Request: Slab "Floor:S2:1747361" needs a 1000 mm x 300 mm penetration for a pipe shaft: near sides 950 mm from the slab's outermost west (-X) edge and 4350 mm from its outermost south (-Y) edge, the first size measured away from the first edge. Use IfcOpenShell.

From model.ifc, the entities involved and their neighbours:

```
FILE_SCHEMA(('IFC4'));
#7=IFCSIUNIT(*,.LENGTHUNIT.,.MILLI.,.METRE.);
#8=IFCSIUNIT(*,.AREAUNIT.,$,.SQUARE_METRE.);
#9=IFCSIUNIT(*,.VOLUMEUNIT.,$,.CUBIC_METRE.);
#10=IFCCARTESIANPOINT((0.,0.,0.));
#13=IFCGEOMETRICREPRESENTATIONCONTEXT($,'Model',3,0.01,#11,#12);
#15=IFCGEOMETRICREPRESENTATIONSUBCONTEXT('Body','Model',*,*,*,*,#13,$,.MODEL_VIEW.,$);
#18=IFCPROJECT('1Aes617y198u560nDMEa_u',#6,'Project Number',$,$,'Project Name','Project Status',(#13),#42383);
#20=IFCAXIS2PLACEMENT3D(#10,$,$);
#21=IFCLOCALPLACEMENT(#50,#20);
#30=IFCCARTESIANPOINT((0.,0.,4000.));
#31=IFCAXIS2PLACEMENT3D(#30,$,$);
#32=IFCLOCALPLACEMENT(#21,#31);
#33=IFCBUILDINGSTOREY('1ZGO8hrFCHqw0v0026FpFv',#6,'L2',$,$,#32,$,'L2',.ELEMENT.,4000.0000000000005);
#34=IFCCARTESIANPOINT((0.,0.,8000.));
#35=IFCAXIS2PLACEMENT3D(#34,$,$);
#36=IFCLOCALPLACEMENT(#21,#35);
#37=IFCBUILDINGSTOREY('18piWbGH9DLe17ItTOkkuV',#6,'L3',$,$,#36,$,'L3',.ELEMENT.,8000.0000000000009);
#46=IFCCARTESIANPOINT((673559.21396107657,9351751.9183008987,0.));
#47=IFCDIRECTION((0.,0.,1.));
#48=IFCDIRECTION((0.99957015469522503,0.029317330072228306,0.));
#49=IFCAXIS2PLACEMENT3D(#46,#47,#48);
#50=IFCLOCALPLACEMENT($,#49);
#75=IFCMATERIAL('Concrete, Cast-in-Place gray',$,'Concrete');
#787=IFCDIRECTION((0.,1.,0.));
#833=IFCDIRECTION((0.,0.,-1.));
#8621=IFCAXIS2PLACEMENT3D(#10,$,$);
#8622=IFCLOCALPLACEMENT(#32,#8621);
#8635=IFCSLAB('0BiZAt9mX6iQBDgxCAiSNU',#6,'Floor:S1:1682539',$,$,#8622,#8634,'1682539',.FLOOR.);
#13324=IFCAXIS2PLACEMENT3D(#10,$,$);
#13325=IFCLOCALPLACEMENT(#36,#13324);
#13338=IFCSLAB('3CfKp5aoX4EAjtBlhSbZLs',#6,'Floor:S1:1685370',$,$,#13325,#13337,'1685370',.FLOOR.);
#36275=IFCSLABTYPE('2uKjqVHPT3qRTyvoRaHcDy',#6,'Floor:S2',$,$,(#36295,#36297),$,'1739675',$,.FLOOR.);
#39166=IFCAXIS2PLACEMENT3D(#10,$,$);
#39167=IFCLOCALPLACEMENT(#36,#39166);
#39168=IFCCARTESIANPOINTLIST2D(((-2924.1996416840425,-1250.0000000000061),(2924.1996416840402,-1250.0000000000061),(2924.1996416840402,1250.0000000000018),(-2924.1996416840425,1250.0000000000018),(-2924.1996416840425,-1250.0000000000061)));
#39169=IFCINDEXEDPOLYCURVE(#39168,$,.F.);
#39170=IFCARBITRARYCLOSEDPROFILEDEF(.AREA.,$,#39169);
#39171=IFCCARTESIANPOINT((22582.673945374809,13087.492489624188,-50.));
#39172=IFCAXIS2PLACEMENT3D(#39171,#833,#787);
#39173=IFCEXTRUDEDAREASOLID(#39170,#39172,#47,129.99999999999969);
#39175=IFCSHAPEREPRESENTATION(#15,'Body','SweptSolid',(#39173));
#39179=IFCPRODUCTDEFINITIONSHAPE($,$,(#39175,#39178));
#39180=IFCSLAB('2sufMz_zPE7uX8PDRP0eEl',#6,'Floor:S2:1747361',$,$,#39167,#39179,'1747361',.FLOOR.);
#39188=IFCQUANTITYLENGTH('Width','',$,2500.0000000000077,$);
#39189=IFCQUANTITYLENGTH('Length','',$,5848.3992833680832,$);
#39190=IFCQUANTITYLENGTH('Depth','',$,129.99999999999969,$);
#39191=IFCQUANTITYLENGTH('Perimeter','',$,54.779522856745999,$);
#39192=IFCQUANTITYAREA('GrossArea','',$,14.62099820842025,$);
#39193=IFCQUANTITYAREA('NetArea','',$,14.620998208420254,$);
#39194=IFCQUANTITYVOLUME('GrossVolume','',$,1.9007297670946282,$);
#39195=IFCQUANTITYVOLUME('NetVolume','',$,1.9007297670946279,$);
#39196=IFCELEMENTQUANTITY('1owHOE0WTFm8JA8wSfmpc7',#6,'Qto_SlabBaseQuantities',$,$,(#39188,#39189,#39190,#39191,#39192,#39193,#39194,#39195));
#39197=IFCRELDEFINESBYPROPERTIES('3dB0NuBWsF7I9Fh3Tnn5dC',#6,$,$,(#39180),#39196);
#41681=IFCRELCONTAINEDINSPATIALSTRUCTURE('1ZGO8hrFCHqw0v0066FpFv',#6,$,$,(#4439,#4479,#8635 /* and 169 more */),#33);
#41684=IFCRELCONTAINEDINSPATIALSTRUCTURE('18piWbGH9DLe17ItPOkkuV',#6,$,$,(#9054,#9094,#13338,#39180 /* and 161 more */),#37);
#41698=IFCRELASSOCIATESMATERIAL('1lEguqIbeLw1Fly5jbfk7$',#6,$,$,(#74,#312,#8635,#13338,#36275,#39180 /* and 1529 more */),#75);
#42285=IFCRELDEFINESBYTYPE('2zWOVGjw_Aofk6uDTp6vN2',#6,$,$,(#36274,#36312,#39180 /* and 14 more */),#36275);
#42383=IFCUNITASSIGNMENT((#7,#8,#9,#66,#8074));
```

```python
import numpy as np
import ifcopenshell
import ifcopenshell.api.feature
import ifcopenshell.api.geometry
import ifcopenshell.api.pset
import ifcopenshell.api.root
import ifcopenshell.geom
import ifcopenshell.util.element
import ifcopenshell.util.placement
import ifcopenshell.util.representation
import ifcopenshell.util.shape
import ifcopenshell.util.unit

model = ifcopenshell.open("model.ifc")
unit_scale = ifcopenshell.util.unit.calculate_unit_scale(model)
area_scale = ifcopenshell.util.unit.calculate_unit_scale(model, "AREAUNIT")
volume_scale = ifcopenshell.util.unit.calculate_unit_scale(model, "VOLUMEUNIT")
settings = ifcopenshell.geom.settings()


def volume(element):
    """Net volume in cubic metres, openings subtracted."""
    shape = ifcopenshell.geom.create_shape(settings, element)
    return ifcopenshell.util.shape.get_volume(shape.geometry)


slab = model.by_guid("2sufMz_zPE7uX8PDRP0eEl")
before = volume(slab)

# Extent in the slab's own axes, in metres. The edges named are its -X and -Y sides.
slab_shape = ifcopenshell.geom.create_shape(settings, slab)
vertices = ifcopenshell.util.shape.get_vertices(slab_shape.geometry)
x_min, y_min, bottom = vertices.min(axis=0)
top = vertices[:, 2].max()

opening = ifcopenshell.api.root.create_entity(model, ifc_class="IfcOpeningElement", name="Pipe shaft opening", predefined_type="OPENING")
context = ifcopenshell.util.representation.get_context(model, "Model", "Body", "MODEL_VIEW")
width, depth = 1, 0.3
outline = [(0.0, 0.0), (width, 0.0), (width, depth), (0.0, depth), (0.0, 0.0)]
# Overshoot both faces by 50 mm so the cut is clean.
shape = ifcopenshell.api.geometry.add_slab_representation(
    model, context=context, depth=top - bottom + 0.1, polyline=outline
)
ifcopenshell.api.geometry.assign_representation(model, product=opening, representation=shape)

matrix = ifcopenshell.util.placement.get_local_placement(slab.ObjectPlacement)
matrix[:, 3] = matrix @ np.append(np.array([x_min + 0.95, y_min + 4.35, bottom - 0.05]) / unit_scale, 1.0)
ifcopenshell.api.geometry.edit_object_placement(model, product=opening, matrix=matrix, is_si=False)
ifcopenshell.api.feature.add_feature(model, feature=opening, element=slab)

after = volume(slab)

# Update the slab's stored quantities.
qto = model.by_id(ifcopenshell.util.element.get_pset(slab, "Qto_SlabBaseQuantities", should_inherit=False)["id"])
ifcopenshell.api.pset.edit_qto(model, qto=qto, properties={
    "NetArea": after / (top - bottom) / area_scale,
    "NetVolume": after / volume_scale,
})

print(f"slab volume {before:.3f} -> {after:.3f} m3")

model.write("model-out.ifc")
```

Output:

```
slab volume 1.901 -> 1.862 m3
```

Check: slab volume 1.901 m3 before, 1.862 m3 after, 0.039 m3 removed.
